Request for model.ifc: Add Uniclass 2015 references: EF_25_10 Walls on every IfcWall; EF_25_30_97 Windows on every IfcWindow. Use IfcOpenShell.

First a look at what the model holds.

```python
import ifcopenshell

model = ifcopenshell.open("model.ifc")
print(model.schema)
print("classifications:", [c.Name for c in model.by_type("IfcClassification")])
for ifc_class in ("IfcDoor", "IfcRoof", "IfcStair", "IfcWall", "IfcWindow"):
    print(ifc_class, len(model.by_type(ifc_class)))
```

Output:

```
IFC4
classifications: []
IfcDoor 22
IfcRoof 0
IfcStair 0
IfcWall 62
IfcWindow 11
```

```python
import ifcopenshell
import ifcopenshell.api.classification

model = ifcopenshell.open("model.ifc")

system = ifcopenshell.api.classification.add_classification(model, classification="Uniclass 2015")

codes = {
    "IfcWall": ("EF_25_10", "Walls"),
    "IfcWindow": ("EF_25_30_97", "Windows"),
}
for ifc_class, (code, name) in codes.items():
    products = model.by_type(ifc_class)
    ifcopenshell.api.classification.add_reference(
        model, products=products, classification=system, identification=code, name=name
    )
    print(code, len(products))

model.write("model-out.ifc")
```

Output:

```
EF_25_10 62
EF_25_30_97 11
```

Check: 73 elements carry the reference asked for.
